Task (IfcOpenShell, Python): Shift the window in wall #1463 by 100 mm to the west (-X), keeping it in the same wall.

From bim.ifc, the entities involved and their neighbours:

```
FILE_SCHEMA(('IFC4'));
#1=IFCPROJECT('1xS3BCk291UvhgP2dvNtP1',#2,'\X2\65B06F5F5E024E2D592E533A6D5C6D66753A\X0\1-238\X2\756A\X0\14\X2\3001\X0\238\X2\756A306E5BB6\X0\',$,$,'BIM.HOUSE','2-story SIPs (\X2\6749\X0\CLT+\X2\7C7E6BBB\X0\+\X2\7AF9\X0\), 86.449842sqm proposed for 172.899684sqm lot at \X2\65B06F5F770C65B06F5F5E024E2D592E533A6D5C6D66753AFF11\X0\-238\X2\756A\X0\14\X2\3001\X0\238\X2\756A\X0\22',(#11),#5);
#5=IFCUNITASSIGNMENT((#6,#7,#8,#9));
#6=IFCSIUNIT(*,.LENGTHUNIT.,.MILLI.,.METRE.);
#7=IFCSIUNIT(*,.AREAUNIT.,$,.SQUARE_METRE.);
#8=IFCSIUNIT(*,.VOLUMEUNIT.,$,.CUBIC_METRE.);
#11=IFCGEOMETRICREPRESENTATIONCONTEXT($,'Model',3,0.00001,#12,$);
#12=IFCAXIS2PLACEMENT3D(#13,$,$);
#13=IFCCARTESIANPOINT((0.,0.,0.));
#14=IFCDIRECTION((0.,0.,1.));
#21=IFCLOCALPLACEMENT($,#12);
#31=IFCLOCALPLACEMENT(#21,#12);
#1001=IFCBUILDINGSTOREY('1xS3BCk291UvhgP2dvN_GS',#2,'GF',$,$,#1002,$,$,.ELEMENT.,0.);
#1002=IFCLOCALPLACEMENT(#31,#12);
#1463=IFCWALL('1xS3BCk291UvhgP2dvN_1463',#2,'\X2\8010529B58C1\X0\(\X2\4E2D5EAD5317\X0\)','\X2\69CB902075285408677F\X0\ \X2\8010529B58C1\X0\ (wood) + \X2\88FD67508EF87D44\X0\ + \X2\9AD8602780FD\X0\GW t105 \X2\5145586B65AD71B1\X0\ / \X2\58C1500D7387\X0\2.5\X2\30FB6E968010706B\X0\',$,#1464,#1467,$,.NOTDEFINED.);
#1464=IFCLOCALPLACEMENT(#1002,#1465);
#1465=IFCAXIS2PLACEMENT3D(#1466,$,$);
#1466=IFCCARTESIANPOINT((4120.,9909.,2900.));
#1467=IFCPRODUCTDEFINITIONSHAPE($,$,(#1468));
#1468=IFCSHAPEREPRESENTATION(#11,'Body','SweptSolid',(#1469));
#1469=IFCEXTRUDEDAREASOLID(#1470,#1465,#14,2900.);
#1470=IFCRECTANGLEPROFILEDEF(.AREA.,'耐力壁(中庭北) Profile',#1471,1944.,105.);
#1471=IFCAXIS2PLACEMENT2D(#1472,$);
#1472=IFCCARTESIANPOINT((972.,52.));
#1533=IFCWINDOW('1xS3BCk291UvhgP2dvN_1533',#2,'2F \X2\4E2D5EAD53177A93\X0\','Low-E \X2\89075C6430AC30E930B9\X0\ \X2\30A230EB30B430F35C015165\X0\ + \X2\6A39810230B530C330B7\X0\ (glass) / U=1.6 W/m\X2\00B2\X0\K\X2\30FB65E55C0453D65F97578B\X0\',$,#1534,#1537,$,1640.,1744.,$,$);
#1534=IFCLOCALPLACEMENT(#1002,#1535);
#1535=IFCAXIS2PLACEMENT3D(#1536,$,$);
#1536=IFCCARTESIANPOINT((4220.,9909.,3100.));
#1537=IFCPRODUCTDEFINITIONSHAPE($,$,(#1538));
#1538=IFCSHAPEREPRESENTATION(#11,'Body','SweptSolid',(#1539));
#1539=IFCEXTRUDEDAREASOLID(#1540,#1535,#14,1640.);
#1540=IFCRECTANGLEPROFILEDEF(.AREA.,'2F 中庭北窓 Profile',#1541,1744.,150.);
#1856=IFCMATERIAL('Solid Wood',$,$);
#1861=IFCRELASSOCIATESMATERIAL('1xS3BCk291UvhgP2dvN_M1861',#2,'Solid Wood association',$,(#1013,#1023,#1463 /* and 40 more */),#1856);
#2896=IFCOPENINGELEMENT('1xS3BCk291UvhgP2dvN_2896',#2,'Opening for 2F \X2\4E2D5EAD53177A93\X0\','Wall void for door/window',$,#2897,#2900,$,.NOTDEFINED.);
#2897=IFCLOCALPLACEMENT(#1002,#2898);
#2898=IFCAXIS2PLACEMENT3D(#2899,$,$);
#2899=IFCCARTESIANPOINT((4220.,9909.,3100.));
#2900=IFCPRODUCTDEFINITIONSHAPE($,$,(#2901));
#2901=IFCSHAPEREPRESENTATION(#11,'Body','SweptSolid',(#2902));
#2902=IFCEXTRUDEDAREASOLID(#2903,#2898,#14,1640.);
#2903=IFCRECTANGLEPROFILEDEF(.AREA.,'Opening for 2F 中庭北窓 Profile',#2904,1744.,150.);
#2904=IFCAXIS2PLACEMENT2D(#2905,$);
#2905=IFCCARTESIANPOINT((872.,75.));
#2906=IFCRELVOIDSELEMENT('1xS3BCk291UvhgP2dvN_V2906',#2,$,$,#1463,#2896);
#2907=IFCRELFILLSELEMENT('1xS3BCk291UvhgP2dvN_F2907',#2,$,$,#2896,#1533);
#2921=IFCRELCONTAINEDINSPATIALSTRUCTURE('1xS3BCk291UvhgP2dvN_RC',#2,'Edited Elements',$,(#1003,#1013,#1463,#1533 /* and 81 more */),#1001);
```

```python
import ifcopenshell
import ifcopenshell.api.geometry
import ifcopenshell.util.placement
import ifcopenshell.util.unit

model = ifcopenshell.open("bim.ifc")
unit_scale = ifcopenshell.util.unit.calculate_unit_scale(model)

window = model.by_id(1533)
opening = window.FillsVoids[0].RelatingOpeningElement
wall = opening.VoidsElements[0].RelatingBuildingElement

wall_matrix = ifcopenshell.util.placement.get_local_placement(wall.ObjectPlacement)
shift = wall_matrix[:3, 0] * -0.1 / unit_scale
before = ifcopenshell.util.placement.get_local_placement(window.ObjectPlacement)[:3, 3].copy()

# The window is not placed relative to its opening, so move both.
for product in (opening, window):
    matrix = ifcopenshell.util.placement.get_local_placement(product.ObjectPlacement)
    matrix[:3, 3] += shift
    ifcopenshell.api.geometry.edit_object_placement(model, product=product, matrix=matrix, is_si=False)

after = ifcopenshell.util.placement.get_local_placement(window.ObjectPlacement)[:3, 3]
print("window moved by", (after - before).round(3) + 0.0)

model.write("bim_edited.ifc")
```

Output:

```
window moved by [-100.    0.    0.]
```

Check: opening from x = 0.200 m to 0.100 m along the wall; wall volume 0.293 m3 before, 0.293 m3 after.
